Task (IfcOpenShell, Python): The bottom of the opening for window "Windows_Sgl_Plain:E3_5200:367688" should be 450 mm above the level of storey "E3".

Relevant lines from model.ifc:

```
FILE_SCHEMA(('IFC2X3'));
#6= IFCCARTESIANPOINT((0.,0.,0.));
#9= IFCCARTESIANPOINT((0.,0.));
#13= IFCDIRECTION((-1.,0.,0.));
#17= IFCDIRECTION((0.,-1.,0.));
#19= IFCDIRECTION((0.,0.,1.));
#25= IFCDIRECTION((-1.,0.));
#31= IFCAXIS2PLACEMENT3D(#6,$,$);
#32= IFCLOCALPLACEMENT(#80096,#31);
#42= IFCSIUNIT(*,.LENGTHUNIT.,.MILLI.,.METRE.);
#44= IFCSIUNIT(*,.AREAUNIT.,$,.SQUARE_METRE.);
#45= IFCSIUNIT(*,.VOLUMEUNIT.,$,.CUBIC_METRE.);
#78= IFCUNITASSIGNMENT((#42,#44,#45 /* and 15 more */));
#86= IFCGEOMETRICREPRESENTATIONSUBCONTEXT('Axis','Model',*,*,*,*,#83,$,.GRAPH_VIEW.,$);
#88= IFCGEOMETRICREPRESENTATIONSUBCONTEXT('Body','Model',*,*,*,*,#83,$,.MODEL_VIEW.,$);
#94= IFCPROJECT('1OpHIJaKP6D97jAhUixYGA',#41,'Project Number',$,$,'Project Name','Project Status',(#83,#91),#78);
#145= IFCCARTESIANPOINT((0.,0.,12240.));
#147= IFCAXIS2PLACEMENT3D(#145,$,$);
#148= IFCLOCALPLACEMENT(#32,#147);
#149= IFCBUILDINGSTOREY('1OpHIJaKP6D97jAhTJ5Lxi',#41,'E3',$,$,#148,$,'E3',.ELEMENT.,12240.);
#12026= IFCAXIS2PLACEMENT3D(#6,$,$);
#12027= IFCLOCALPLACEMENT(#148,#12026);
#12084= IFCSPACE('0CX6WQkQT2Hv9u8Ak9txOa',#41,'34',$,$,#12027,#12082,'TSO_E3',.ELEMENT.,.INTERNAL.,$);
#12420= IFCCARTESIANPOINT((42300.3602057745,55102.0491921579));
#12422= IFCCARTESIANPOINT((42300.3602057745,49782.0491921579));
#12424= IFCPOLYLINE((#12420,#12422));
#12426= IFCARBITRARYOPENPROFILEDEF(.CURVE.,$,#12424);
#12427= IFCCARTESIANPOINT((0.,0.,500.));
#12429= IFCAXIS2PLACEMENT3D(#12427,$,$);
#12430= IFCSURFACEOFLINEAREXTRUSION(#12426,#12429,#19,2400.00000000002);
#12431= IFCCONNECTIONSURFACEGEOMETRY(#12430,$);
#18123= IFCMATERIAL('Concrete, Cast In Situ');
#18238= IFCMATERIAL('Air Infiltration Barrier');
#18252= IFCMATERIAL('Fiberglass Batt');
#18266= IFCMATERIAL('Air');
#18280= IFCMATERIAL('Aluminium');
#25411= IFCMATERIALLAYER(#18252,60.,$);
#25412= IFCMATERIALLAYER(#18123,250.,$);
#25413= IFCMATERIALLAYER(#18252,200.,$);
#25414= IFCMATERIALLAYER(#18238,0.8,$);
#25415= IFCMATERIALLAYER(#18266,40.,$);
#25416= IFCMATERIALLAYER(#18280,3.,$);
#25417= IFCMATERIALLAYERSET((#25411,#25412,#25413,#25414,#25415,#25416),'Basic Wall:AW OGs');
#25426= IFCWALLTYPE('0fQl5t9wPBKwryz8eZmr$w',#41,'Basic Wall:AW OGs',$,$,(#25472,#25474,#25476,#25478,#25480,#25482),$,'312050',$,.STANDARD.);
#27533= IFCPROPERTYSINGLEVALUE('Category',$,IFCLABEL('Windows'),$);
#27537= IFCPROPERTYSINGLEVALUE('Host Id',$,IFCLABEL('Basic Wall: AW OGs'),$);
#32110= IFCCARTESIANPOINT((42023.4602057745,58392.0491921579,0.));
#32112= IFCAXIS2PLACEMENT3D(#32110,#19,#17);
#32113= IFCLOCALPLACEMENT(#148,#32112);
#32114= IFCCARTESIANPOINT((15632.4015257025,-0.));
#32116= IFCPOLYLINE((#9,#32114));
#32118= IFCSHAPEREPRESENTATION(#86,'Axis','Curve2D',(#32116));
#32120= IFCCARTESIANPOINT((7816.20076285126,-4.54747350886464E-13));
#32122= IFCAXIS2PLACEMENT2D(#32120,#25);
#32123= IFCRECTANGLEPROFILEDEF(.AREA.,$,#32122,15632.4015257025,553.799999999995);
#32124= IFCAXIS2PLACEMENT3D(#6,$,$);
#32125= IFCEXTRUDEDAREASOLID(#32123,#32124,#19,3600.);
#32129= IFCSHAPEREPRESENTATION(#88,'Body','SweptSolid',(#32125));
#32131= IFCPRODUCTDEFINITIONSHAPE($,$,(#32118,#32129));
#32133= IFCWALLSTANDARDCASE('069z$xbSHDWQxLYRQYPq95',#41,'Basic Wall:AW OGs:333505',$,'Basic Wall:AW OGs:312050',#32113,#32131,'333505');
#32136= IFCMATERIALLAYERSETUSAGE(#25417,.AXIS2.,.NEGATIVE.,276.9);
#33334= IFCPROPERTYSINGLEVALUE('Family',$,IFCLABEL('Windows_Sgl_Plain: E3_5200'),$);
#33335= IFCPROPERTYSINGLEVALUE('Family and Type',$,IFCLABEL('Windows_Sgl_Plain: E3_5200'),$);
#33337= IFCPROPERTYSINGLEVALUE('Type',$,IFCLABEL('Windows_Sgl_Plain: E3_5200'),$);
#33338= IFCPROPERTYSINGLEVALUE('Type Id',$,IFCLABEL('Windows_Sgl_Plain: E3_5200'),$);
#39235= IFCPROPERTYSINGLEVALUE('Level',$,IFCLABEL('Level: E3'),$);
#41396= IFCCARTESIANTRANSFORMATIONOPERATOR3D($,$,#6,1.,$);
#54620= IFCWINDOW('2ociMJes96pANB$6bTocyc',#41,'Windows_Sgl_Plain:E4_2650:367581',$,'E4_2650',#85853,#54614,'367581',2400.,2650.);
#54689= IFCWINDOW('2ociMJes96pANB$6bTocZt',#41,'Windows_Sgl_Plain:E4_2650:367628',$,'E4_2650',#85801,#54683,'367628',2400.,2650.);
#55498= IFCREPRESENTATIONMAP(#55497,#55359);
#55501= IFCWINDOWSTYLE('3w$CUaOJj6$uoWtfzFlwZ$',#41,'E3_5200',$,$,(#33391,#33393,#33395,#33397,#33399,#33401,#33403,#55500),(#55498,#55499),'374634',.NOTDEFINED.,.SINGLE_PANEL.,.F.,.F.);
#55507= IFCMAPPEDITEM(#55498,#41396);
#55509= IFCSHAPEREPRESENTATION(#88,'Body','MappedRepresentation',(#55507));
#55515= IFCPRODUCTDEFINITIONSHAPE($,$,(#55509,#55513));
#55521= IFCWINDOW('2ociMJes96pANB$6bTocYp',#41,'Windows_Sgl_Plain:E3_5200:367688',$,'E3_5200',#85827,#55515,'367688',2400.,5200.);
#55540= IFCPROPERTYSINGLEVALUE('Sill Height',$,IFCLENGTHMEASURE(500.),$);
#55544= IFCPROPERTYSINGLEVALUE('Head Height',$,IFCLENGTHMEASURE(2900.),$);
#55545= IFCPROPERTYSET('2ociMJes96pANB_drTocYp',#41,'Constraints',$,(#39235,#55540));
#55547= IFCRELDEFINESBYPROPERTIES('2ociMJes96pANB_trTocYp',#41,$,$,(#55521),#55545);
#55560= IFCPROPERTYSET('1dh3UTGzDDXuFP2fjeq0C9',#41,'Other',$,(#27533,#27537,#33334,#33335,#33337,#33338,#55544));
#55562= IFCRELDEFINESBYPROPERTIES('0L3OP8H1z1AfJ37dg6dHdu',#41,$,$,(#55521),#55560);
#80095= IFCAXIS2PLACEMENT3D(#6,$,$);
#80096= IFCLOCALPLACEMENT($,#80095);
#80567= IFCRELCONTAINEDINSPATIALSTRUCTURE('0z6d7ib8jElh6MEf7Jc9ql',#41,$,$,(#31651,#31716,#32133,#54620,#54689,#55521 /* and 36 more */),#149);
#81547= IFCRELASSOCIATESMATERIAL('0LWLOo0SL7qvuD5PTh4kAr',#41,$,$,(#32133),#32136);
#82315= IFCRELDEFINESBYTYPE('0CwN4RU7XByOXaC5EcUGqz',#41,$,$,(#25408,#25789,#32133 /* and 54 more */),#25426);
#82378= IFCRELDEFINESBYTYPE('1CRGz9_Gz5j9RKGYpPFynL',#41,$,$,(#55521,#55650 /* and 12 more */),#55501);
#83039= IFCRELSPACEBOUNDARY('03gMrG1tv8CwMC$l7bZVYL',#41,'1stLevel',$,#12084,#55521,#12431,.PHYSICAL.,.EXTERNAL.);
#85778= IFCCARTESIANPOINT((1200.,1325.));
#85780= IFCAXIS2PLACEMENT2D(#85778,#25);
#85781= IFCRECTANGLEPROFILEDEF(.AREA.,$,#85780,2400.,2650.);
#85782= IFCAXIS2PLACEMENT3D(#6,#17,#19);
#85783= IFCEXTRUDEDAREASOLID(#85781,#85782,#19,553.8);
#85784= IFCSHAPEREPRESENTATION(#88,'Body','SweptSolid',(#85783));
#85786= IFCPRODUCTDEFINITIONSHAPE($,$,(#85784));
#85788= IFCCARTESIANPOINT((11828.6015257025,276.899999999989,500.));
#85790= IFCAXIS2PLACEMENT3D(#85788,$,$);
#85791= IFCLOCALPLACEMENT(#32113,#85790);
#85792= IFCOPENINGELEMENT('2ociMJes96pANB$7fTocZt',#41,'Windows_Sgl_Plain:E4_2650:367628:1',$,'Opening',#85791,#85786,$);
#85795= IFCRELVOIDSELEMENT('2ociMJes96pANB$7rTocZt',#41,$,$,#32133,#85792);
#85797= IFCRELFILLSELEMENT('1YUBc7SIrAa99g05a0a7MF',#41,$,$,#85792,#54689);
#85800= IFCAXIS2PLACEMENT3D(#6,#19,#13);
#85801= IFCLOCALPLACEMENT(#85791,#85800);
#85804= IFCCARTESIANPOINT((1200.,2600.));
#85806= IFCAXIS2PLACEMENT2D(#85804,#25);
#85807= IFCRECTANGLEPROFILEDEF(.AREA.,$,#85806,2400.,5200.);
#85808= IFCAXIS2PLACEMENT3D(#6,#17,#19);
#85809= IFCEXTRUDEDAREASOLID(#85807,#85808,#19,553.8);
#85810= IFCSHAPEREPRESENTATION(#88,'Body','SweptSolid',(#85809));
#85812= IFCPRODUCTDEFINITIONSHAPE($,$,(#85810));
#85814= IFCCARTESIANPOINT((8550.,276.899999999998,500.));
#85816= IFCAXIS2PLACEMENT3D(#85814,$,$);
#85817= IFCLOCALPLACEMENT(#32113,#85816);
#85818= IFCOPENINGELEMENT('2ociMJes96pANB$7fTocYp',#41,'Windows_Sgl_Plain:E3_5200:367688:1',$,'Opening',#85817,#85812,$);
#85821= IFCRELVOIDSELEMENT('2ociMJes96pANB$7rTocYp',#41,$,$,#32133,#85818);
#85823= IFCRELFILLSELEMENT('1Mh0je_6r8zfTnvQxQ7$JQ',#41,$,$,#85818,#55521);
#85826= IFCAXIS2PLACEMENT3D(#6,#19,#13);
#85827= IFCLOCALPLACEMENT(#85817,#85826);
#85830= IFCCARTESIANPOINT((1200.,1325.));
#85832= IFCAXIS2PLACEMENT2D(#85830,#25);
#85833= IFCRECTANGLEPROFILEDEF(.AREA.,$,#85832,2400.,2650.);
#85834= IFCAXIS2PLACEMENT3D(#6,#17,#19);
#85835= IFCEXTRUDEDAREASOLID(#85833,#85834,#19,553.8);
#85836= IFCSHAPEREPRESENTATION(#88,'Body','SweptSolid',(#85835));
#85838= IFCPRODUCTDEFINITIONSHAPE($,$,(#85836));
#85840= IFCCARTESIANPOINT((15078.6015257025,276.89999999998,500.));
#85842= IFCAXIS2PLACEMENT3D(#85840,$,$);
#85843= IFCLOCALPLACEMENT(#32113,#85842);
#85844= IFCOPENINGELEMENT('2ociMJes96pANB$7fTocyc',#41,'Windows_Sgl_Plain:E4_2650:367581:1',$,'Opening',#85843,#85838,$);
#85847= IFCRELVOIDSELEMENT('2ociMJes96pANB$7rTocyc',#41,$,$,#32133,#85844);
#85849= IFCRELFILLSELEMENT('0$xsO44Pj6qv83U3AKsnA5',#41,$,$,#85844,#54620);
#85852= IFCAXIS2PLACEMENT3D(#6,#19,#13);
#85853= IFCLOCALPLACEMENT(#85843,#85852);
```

```python
import numpy as np
import ifcopenshell
import ifcopenshell.api.geometry
import ifcopenshell.api.pset
import ifcopenshell.geom
import ifcopenshell.util.element
import ifcopenshell.util.placement
import ifcopenshell.util.shape
import ifcopenshell.util.unit

model = ifcopenshell.open("model.ifc")
unit_scale = ifcopenshell.util.unit.calculate_unit_scale(model)

window = model.by_id(55521)
opening = window.FillsVoids[0].RelatingOpeningElement
storey = ifcopenshell.util.element.get_container(window, ifc_class="IfcBuildingStorey")
level = ifcopenshell.util.placement.get_local_placement(storey.ObjectPlacement)[2, 3]

# The opening's origin need not be at the sill, so measure its lowest point.
shape = ifcopenshell.geom.create_shape(ifcopenshell.geom.settings(), opening)
bottom = ifcopenshell.util.shape.get_shape_bottom_elevation(shape, shape.geometry) / unit_scale
dz = level + 0.45 / unit_scale - bottom

shift = np.array([0.0, 0.0, dz])
# The window is placed relative to its opening, so it follows when the opening moves.
matrix = ifcopenshell.util.placement.get_local_placement(opening.ObjectPlacement)
matrix[:3, 3] += shift
ifcopenshell.api.geometry.edit_object_placement(
    model, product=opening, matrix=matrix, is_si=False, should_transform_children=True
)

# Space boundary surfaces are stored in each space's coordinates; move them too.
for rel in window.ProvidesBoundaries:
    if not rel.ConnectionGeometry:
        continue
    surface = rel.ConnectionGeometry.SurfaceOnRelatingElement
    space_matrix = ifcopenshell.util.placement.get_local_placement(rel.RelatingSpace.ObjectPlacement)
    point = np.array(surface.Position.Location.Coordinates) + space_matrix[:3, :3].T @ shift
    surface.Position = model.createIfcAxis2Placement3D(
        model.createIfcCartesianPoint(point.tolist()), surface.Position.Axis, surface.Position.RefDirection
    )

# Keep the stored heights in step.
pset = model.by_id(ifcopenshell.util.element.get_pset(window, "Constraints", should_inherit=False)["id"])
ifcopenshell.api.pset.edit_pset(model, pset=pset, properties={
    "Sill Height": model.create_entity("IfcLengthMeasure", ifcopenshell.util.element.get_pset(window, "Constraints", "Sill Height") + dz),
})
pset = model.by_id(ifcopenshell.util.element.get_pset(window, "Other", should_inherit=False)["id"])
ifcopenshell.api.pset.edit_pset(model, pset=pset, properties={
    "Head Height": model.create_entity("IfcLengthMeasure", ifcopenshell.util.element.get_pset(window, "Other", "Head Height") + dz),
})

print(f"moved by {dz * unit_scale:+.3f} m")

model.write("model_edited.ifc")
```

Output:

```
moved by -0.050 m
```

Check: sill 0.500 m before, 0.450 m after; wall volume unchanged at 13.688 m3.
